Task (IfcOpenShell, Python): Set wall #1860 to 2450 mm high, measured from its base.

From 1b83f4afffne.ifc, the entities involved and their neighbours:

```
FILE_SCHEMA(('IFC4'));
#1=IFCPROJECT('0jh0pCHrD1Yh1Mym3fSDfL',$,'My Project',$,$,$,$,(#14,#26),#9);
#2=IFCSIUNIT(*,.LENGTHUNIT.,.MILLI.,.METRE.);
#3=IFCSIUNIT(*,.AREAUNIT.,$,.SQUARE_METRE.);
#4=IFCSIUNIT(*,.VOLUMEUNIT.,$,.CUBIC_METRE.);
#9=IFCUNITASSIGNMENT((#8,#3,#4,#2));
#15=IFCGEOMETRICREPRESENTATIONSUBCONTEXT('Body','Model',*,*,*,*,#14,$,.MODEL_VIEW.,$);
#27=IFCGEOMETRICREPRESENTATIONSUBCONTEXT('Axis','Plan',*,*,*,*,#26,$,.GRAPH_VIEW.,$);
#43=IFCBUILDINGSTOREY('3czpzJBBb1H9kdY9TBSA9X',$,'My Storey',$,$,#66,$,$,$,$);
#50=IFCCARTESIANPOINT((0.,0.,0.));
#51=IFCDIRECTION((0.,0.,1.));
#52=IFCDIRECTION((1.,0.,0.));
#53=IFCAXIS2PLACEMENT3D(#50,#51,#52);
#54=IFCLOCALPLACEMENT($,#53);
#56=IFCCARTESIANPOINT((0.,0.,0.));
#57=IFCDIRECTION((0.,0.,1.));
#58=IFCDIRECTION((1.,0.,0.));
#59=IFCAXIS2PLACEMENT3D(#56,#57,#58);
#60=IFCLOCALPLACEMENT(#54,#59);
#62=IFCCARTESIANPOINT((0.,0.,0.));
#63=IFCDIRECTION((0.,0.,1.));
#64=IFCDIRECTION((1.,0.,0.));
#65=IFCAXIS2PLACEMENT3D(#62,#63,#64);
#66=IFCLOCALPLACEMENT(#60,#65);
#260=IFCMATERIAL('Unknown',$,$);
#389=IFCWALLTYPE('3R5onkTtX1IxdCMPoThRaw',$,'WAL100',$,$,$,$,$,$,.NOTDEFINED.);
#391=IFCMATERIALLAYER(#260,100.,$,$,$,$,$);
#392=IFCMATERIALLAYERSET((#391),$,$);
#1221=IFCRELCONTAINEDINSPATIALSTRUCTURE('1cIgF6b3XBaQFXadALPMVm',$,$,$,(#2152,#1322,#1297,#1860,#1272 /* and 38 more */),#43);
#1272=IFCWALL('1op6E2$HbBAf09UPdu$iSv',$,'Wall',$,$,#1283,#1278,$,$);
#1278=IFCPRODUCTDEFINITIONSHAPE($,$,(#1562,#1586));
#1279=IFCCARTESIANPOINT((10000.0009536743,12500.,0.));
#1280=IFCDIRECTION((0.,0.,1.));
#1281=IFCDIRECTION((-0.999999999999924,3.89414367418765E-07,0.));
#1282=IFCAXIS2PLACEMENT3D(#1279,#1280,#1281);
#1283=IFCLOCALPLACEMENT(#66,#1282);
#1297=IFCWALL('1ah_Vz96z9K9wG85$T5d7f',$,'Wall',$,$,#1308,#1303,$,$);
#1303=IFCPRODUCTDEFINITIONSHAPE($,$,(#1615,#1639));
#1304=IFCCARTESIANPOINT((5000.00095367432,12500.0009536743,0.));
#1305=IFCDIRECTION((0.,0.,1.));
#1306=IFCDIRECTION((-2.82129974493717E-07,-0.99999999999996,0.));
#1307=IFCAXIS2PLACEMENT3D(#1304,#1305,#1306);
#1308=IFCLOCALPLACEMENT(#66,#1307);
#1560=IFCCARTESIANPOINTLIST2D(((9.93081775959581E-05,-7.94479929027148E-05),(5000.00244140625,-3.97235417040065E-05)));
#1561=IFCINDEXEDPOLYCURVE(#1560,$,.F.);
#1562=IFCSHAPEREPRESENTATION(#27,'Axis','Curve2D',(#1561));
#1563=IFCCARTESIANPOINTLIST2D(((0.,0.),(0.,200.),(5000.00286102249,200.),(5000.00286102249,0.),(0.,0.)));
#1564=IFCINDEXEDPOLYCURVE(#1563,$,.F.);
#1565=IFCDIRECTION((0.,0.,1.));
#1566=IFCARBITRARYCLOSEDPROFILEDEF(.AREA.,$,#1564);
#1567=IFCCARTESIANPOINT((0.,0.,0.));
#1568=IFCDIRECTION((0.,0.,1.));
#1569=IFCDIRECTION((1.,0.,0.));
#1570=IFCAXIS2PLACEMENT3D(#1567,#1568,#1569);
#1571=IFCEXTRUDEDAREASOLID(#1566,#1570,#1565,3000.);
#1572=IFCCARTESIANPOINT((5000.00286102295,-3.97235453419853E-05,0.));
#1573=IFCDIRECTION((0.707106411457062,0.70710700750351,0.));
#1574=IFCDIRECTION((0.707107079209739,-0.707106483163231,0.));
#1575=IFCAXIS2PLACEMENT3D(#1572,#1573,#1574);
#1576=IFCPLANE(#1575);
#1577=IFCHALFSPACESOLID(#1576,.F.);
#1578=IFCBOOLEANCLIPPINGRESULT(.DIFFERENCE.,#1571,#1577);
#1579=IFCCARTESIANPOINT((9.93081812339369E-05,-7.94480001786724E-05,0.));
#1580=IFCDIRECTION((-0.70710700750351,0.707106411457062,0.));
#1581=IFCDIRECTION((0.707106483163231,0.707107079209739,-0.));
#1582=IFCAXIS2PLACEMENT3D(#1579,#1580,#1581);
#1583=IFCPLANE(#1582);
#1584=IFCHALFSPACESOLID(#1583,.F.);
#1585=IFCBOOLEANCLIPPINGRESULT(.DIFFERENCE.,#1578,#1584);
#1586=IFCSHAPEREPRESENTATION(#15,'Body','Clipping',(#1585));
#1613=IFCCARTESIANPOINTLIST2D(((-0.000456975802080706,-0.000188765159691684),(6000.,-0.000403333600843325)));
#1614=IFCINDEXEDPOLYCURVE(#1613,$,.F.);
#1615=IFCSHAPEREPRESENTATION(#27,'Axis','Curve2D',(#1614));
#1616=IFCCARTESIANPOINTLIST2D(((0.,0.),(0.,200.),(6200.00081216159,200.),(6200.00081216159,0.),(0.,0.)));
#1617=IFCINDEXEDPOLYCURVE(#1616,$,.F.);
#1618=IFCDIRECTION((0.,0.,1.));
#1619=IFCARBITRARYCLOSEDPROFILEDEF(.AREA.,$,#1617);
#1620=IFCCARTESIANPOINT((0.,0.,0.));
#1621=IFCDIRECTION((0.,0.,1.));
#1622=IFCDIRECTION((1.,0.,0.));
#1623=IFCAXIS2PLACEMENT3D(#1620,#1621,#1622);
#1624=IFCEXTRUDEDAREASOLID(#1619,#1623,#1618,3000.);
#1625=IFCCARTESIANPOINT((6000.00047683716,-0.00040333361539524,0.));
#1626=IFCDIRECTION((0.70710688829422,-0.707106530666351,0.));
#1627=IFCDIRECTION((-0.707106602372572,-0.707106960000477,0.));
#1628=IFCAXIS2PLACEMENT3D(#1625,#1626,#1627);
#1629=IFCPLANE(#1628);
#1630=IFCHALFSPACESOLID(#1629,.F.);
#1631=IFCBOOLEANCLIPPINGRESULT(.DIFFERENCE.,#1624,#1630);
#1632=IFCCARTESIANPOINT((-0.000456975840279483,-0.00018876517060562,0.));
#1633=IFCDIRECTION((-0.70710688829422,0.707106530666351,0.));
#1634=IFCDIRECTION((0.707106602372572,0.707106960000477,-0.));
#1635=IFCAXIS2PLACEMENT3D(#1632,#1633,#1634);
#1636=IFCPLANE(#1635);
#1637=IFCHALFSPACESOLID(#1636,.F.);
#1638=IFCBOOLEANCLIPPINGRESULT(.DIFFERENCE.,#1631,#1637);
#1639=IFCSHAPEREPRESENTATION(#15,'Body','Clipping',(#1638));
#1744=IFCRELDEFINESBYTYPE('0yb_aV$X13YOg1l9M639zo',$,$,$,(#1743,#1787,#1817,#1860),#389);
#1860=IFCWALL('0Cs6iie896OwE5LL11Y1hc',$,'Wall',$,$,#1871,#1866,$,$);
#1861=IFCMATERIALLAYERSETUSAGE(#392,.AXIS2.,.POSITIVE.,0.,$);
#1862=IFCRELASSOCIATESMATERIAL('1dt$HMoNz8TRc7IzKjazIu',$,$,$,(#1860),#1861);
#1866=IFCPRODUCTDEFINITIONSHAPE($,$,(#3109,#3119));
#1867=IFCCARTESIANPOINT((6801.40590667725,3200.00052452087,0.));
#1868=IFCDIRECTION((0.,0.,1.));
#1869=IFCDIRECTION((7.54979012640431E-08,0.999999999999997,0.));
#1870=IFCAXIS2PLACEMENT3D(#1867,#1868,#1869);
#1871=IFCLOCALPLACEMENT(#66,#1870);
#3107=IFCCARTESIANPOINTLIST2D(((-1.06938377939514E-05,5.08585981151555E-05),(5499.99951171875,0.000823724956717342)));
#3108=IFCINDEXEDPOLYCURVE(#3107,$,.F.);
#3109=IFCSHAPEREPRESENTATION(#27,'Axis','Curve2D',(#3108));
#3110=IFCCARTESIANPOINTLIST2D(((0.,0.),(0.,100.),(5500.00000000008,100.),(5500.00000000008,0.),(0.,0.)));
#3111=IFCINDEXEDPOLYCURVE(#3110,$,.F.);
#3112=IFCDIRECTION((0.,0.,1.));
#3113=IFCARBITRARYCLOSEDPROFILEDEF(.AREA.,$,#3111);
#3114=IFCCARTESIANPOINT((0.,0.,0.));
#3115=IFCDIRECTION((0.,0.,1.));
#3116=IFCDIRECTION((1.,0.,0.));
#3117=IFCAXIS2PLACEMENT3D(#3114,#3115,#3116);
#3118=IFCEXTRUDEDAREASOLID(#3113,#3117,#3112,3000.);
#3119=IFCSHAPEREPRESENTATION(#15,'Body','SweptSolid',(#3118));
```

```python
import ifcopenshell
import ifcopenshell.geom
import ifcopenshell.util.representation
import ifcopenshell.util.shape

model = ifcopenshell.open("1b83f4afffne.ifc")
settings = ifcopenshell.geom.settings()


def volume(element):
    """Net volume in cubic metres, openings subtracted."""
    shape = ifcopenshell.geom.create_shape(settings, element)
    return ifcopenshell.util.shape.get_volume(shape.geometry)


wall = model.by_id(1860)
before = volume(wall)

body = ifcopenshell.util.representation.get_representation(wall, "Model", "Body")
solid = body.Items[0]
old_height = solid.Depth
solid.Depth = 2450.0
after = volume(wall)

print(f"height {old_height:g} -> {solid.Depth:g}, volume {before:.3f} -> {after:.3f} m3")

model.write("1b83f4afffne_edited.ifc")
```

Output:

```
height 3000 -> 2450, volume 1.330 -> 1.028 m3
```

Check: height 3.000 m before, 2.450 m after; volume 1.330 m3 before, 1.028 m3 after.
